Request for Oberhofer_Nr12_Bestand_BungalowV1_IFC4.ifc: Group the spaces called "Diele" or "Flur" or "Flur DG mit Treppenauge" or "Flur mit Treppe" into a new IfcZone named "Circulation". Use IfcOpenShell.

First a look at what the model holds.

```python
import ifcopenshell

model = ifcopenshell.open("Oberhofer_Nr12_Bestand_BungalowV1_IFC4.ifc")
print(model.schema)
seen = {}
for space in model.by_type("IfcSpace"):
    seen[space.LongName] = seen.get(space.LongName, 0) + 1
for name, count in sorted(seen.items(), key=str):
    print(count, "x", name)
print("zones:", [z.Name for z in model.by_type("IfcZone")][:20])
```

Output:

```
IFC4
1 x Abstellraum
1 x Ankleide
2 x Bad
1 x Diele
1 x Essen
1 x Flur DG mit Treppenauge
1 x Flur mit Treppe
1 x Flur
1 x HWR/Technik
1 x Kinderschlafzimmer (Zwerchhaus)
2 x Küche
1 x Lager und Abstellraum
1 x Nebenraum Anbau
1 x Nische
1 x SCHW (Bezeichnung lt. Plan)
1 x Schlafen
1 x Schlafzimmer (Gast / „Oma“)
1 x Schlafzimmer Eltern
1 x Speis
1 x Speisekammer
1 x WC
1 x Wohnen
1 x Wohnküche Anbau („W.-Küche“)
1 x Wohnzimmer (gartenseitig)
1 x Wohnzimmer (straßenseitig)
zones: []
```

```python
import ifcopenshell
import ifcopenshell.api.group
import ifcopenshell.api.root

model = ifcopenshell.open("Oberhofer_Nr12_Bestand_BungalowV1_IFC4.ifc")

names = {"Diele", "Flur", "Flur DG mit Treppenauge", "Flur mit Treppe"}
spaces = [s for s in model.by_type("IfcSpace") if s.LongName in names]

zone = ifcopenshell.api.root.create_entity(model, ifc_class="IfcZone", name="Circulation")
ifcopenshell.api.group.assign_group(model, products=spaces, group=zone)
print(len(spaces), "spaces in", zone.Name)

model.write("Oberhofer_Nr12_Bestand_BungalowV1_IFC4_edited.ifc")
```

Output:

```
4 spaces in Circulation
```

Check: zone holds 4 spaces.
